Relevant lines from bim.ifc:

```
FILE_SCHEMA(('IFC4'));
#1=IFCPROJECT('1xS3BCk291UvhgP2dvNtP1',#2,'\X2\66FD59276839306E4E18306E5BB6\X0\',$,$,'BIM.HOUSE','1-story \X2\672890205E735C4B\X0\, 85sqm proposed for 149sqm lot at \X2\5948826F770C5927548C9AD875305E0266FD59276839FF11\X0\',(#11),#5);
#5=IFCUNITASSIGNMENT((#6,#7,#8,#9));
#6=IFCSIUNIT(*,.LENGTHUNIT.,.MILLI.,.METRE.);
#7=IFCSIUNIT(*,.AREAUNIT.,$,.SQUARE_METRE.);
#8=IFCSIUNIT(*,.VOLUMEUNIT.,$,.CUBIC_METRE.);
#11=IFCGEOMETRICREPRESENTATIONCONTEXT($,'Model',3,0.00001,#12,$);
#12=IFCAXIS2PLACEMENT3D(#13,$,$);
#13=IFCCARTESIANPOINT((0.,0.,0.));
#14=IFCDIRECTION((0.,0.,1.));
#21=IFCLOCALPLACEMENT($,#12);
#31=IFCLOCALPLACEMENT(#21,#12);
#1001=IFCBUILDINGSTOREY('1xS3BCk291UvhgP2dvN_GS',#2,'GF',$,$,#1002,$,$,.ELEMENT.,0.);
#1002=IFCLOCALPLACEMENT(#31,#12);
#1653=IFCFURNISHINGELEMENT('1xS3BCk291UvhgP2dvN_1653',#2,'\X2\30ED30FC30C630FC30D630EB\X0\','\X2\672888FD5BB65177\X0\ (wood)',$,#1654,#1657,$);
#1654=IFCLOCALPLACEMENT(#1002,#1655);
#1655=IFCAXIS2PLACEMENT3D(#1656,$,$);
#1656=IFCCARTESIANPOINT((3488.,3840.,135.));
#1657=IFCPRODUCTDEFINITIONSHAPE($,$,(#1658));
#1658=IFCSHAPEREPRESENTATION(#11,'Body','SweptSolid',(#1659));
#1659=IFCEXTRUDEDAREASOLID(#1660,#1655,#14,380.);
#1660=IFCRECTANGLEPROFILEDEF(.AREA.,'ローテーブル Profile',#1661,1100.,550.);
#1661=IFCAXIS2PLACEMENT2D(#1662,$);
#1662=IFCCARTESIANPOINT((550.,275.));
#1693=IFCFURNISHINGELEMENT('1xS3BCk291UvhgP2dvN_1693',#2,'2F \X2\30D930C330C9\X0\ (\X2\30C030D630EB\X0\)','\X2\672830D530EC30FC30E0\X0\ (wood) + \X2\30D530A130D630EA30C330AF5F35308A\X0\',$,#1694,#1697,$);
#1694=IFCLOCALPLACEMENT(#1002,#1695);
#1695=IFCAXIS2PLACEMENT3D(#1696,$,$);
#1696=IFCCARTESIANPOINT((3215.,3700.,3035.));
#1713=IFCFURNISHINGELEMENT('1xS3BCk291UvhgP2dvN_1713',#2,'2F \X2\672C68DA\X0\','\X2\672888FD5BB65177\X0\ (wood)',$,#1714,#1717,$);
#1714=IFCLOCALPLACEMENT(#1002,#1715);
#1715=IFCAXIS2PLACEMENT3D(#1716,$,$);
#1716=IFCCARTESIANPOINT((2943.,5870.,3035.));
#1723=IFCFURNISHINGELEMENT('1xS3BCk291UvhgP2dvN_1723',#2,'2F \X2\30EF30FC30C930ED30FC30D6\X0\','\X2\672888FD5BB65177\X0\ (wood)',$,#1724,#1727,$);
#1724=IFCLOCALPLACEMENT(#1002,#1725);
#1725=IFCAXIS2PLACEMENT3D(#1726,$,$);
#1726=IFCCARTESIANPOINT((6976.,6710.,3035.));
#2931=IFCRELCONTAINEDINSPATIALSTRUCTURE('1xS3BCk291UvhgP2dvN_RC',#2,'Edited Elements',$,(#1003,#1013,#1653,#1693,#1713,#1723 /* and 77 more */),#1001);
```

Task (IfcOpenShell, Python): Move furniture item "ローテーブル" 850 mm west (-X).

```python
import ifcopenshell
import ifcopenshell.api.geometry
import ifcopenshell.util.placement

model = ifcopenshell.open("bim.ifc")

item = model.by_guid("1xS3BCk291UvhgP2dvN_1653")
matrix = ifcopenshell.util.placement.get_local_placement(item.ObjectPlacement)
matrix[0, 3] -= 850.0
ifcopenshell.api.geometry.edit_object_placement(model, product=item, matrix=matrix, is_si=False)

print(ifcopenshell.util.placement.get_local_placement(item.ObjectPlacement).round(3) + 0.0)

model.write("bim_edited.ifc")
```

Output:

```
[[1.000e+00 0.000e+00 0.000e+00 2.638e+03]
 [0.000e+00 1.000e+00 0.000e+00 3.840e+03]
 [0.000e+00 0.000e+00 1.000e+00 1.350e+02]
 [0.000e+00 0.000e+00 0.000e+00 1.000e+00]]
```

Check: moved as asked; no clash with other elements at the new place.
